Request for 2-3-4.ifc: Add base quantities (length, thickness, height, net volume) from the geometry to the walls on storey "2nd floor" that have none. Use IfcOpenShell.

First a look at what the model holds.

```python
import ifcopenshell
import ifcopenshell.util.element
import ifcopenshell.util.unit

model = ifcopenshell.open("2-3-4.ifc")
print(model.schema)
for unit_type in ("LENGTHUNIT", "AREAUNIT", "VOLUMEUNIT"):
    print(unit_type, ifcopenshell.util.unit.calculate_unit_scale(model, unit_type))
storey = next(s for s in model.by_type("IfcBuildingStorey") if s.Name == "2nd floor")
walls = [e for e in ifcopenshell.util.element.get_decomposition(storey) if e.is_a("IfcWall")]
for e in sorted(walls, key=lambda e: e.id()):
    print(e.id(), e.is_a(), e.Name, list(ifcopenshell.util.element.get_psets(e, qtos_only=True)), sep=" | ")
```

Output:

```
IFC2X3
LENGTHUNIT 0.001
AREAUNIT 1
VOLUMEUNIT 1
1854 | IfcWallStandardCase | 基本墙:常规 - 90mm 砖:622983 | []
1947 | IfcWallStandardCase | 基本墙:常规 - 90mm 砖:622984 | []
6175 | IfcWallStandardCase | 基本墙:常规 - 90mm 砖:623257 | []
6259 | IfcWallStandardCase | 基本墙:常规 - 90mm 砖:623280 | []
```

```python
import ifcopenshell
import ifcopenshell.api.pset
import ifcopenshell.geom
import ifcopenshell.util.element
import ifcopenshell.util.shape
import ifcopenshell.util.unit

model = ifcopenshell.open("2-3-4.ifc")
unit_scale = ifcopenshell.util.unit.calculate_unit_scale(model)
volume_scale = ifcopenshell.util.unit.calculate_unit_scale(model, "VOLUMEUNIT")
settings = ifcopenshell.geom.settings()

storey = next(s for s in model.by_type("IfcBuildingStorey") if s.Name == "2nd floor")
walls = [e for e in ifcopenshell.util.element.get_decomposition(storey) if e.is_a("IfcWall")]

for e in sorted(walls, key=lambda e: e.id()):
    if ifcopenshell.util.element.get_psets(e, qtos_only=True, should_inherit=False):
        continue
    # Geometry comes back in metres, in the element's own axes.
    shape = ifcopenshell.geom.create_shape(settings, e)
    values = {
        "Length": ifcopenshell.util.shape.get_x(shape.geometry) / unit_scale,
        "Width": ifcopenshell.util.shape.get_y(shape.geometry) / unit_scale,
        "Height": ifcopenshell.util.shape.get_z(shape.geometry) / unit_scale,
        "NetVolume": ifcopenshell.util.shape.get_volume(shape.geometry) / volume_scale,
    }
    qto = ifcopenshell.api.pset.add_qto(model, product=e, name="BaseQuantities")
    ifcopenshell.api.pset.edit_qto(model, qto=qto, properties=values)
    print(e.id(), {k: round(v, 3) for k, v in values.items()})

model.write("2-3-4_rev.ifc")
```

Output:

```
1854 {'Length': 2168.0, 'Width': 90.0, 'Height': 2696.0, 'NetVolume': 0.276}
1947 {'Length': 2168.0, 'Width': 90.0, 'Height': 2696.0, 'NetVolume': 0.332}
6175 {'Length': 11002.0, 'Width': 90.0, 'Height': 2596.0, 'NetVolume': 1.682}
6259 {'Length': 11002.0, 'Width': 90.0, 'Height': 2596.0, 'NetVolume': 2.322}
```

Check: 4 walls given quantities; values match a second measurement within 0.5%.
